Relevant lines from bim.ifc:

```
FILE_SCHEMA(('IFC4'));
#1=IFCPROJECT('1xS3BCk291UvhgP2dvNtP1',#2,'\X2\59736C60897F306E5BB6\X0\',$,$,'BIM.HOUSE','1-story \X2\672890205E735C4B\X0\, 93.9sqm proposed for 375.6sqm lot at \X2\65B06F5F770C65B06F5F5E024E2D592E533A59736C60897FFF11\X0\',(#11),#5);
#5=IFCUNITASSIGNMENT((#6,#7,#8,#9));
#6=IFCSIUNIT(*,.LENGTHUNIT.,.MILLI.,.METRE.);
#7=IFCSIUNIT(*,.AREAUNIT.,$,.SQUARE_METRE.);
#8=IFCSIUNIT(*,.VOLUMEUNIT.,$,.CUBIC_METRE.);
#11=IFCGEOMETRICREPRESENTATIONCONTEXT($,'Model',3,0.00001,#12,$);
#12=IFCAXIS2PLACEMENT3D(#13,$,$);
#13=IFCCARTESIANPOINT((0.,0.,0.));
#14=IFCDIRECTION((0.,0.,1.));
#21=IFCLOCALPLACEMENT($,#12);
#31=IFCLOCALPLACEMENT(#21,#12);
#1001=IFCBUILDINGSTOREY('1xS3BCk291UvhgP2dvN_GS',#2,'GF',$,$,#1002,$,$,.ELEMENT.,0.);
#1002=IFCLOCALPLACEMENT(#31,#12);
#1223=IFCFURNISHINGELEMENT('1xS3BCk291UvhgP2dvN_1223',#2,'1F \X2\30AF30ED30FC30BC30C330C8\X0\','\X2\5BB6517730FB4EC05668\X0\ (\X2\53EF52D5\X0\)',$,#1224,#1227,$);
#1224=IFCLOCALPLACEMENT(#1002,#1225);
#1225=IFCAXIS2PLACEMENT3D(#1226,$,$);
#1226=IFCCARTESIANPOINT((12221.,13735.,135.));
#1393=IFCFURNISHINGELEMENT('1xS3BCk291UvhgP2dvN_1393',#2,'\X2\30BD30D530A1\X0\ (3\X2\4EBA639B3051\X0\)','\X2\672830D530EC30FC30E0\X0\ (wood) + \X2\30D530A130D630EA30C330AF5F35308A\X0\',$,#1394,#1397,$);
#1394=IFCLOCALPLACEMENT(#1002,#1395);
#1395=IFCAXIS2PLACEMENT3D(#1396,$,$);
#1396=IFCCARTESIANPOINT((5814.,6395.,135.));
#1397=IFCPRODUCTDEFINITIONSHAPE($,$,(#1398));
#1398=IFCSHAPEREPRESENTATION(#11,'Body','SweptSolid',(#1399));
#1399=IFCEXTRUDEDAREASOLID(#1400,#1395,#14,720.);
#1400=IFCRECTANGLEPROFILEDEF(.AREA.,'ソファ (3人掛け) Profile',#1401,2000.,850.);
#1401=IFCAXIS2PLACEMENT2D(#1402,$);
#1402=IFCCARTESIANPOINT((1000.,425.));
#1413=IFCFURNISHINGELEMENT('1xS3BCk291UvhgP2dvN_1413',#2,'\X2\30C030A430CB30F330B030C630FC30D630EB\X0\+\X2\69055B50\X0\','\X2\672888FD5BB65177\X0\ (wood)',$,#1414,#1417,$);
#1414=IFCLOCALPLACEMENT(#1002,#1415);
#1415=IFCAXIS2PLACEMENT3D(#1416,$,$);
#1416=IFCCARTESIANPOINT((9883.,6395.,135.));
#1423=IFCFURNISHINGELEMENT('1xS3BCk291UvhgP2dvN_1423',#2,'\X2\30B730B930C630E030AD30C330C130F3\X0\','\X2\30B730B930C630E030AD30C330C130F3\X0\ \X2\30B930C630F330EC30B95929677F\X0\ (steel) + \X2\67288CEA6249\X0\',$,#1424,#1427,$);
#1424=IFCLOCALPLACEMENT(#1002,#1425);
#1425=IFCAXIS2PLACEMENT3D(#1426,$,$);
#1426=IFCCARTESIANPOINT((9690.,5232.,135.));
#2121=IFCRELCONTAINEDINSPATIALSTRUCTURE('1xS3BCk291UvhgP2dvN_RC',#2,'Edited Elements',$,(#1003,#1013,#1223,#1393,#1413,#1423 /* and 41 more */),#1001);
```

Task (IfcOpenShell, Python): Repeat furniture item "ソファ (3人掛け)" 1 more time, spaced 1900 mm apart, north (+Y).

```python
import numpy as np
import ifcopenshell
import ifcopenshell.api.geometry
import ifcopenshell.api.root
import ifcopenshell.util.element
import ifcopenshell.util.placement

model = ifcopenshell.open("bim.ifc")


def reuse_history(source, copy):
    """copy_class also copies each property set's owner history, people and application; keep the originals."""
    for rel in copy.IsDefinedBy:
        if rel.is_a("IfcRelDefinesByProperties") and (history := rel.RelatingPropertyDefinition.OwnerHistory):
            rel.RelatingPropertyDefinition.OwnerHistory = source.OwnerHistory
            ifcopenshell.util.element.remove_deep2(model, history)


source = model.by_guid("1xS3BCk291UvhgP2dvN_1393")
base = ifcopenshell.util.placement.get_local_placement(source.ObjectPlacement)
step = np.array([0.0, 1.0, 0.0]) * 1900.0

for i in range(1, 2):
    copy = ifcopenshell.api.root.copy_class(model, product=source)
    copy.Representation = ifcopenshell.util.element.copy_deep(
        model, source.Representation, exclude=["IfcGeometricRepresentationContext", "IfcRepresentationMap"]
    )
    reuse_history(source, copy)
    matrix = base.copy()
    matrix[:3, 3] += i * step
    print("added at", matrix[:3, 3].round(3) + 0.0)
    ifcopenshell.api.geometry.edit_object_placement(model, product=copy, matrix=matrix, is_si=False)

model.write("bim-out.ifc")
```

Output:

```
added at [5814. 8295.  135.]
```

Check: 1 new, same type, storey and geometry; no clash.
